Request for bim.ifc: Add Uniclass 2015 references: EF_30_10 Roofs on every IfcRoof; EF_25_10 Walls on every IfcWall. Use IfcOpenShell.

First a look at what the model holds.

```python
import ifcopenshell

model = ifcopenshell.open("bim.ifc")
print(model.schema)
print("classifications:", [c.Name for c in model.by_type("IfcClassification")])
for ifc_class in ("IfcDoor", "IfcRoof", "IfcStair", "IfcWall", "IfcWindow"):
    print(ifc_class, len(model.by_type(ifc_class)))
```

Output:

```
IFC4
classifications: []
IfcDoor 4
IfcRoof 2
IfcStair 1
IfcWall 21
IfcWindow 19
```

```python
import ifcopenshell
import ifcopenshell.api.classification

model = ifcopenshell.open("bim.ifc")

system = ifcopenshell.api.classification.add_classification(model, classification="Uniclass 2015")

codes = {
    "IfcRoof": ("EF_30_10", "Roofs"),
    "IfcWall": ("EF_25_10", "Walls"),
}
for ifc_class, (code, name) in codes.items():
    products = model.by_type(ifc_class)
    ifcopenshell.api.classification.add_reference(
        model, products=products, classification=system, identification=code, name=name
    )
    print(code, len(products))

model.write("bim_v2.ifc")
```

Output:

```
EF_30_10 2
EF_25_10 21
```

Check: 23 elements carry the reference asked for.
